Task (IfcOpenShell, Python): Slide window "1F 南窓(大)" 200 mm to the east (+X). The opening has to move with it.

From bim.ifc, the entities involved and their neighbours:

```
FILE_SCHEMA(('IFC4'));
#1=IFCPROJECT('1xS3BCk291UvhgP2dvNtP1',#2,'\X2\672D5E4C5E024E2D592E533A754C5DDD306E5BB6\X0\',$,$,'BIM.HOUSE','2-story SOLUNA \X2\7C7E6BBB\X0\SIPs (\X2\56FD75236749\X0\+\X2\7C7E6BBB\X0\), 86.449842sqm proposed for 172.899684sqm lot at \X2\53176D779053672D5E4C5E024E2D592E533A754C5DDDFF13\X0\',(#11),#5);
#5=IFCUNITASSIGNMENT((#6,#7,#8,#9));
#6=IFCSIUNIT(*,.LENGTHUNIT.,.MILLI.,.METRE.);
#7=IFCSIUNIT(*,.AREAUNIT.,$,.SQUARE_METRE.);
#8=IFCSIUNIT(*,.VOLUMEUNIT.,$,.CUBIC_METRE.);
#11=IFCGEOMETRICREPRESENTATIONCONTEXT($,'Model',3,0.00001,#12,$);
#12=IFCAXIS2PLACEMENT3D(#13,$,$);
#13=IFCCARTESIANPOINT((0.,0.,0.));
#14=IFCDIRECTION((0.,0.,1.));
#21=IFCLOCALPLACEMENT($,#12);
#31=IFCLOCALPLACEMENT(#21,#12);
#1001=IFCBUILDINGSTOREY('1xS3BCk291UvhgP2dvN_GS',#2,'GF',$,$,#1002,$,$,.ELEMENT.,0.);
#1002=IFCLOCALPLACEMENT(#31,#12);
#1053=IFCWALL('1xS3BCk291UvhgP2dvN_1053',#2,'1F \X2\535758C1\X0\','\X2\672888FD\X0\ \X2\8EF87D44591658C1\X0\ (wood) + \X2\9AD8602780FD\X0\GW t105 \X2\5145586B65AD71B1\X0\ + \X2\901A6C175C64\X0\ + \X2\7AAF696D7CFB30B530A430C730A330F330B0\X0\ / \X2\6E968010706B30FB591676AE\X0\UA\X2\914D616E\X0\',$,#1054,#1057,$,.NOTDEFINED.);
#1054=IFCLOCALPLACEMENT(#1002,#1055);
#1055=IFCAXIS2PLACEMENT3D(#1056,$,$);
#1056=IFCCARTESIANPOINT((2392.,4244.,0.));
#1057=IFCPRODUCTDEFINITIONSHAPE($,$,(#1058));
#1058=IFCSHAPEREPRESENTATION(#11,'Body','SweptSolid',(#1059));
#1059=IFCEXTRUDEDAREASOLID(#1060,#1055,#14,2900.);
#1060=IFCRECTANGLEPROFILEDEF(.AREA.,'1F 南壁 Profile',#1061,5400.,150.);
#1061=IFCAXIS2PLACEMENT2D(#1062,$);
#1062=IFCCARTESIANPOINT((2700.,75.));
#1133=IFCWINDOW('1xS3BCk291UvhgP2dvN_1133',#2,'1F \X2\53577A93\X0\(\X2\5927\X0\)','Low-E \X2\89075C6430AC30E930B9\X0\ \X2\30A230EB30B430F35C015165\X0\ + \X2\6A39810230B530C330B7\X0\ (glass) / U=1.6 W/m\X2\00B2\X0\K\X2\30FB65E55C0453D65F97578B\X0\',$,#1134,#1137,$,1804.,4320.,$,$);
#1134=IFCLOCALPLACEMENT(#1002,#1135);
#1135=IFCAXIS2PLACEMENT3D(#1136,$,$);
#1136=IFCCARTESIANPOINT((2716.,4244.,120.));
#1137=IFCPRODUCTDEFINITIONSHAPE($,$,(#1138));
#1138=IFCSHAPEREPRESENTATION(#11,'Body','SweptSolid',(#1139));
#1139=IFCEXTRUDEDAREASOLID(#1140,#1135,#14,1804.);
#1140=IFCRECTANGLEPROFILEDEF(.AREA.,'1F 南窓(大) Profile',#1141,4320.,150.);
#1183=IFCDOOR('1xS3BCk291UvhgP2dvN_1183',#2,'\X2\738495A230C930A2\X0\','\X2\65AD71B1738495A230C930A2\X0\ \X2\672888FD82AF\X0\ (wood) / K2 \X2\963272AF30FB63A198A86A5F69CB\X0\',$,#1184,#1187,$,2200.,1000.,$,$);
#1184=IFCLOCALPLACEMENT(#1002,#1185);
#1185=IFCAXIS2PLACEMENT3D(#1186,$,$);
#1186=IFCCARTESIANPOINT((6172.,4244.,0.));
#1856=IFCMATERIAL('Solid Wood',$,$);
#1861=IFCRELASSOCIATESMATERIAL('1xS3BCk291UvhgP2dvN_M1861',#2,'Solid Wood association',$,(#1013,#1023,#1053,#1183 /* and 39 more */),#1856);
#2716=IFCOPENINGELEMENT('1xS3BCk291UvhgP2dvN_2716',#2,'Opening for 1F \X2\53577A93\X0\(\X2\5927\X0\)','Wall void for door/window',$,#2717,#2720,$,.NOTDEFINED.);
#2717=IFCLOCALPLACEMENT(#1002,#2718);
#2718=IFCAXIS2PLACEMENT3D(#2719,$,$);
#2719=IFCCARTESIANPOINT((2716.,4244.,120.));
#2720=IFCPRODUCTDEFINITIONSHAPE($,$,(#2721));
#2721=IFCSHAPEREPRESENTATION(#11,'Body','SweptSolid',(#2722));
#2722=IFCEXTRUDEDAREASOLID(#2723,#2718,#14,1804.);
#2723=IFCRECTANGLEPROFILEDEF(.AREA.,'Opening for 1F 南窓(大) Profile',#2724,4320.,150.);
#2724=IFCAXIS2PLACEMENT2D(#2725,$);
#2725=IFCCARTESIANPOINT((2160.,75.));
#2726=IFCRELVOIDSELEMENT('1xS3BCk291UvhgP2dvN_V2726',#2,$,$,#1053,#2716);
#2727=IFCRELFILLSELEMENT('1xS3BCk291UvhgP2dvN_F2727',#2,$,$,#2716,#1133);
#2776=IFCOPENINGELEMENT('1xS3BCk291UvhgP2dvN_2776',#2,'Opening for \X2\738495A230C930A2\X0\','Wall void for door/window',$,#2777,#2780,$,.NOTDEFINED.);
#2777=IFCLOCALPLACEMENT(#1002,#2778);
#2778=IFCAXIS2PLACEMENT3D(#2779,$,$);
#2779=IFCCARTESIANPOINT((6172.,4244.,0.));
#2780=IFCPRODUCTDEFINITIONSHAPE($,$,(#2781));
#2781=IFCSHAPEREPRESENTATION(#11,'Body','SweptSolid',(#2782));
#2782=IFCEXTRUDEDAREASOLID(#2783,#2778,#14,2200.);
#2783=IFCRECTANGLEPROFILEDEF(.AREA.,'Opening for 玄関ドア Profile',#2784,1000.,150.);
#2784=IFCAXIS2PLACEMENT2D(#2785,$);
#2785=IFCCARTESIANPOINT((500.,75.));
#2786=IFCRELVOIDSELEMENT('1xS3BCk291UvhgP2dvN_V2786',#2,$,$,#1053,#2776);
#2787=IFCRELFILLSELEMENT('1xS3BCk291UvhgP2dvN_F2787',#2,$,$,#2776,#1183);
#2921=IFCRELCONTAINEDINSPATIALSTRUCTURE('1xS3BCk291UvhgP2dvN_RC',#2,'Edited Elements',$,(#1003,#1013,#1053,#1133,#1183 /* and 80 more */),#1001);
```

```python
import ifcopenshell
import ifcopenshell.api.geometry
import ifcopenshell.util.placement

model = ifcopenshell.open("bim.ifc")

window = model.by_id(1133)
opening = window.FillsVoids[0].RelatingOpeningElement
wall = opening.VoidsElements[0].RelatingBuildingElement

wall_matrix = ifcopenshell.util.placement.get_local_placement(wall.ObjectPlacement)
shift = wall_matrix[:3, 0] * 200.0
before = ifcopenshell.util.placement.get_local_placement(window.ObjectPlacement)[:3, 3].copy()

# The window is not placed relative to its opening, so move both.
for product in (opening, window):
    matrix = ifcopenshell.util.placement.get_local_placement(product.ObjectPlacement)
    matrix[:3, 3] += shift
    ifcopenshell.api.geometry.edit_object_placement(model, product=product, matrix=matrix, is_si=False)

after = ifcopenshell.util.placement.get_local_placement(window.ObjectPlacement)[:3, 3]
print("window moved by", (after - before).round(3) + 0.0)

model.write("bim-out.ifc")
```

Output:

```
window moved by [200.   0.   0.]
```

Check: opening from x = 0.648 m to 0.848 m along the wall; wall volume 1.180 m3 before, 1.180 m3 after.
